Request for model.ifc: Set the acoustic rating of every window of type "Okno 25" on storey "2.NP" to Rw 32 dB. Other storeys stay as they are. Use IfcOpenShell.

First a look at what the model holds.

```python
import ifcopenshell
import ifcopenshell.util.element

model = ifcopenshell.open("model.ifc")
print(model.schema)
storey = next(s for s in model.by_type("IfcBuildingStorey") if s.Name == "2.NP")
windows = [e for e in ifcopenshell.util.element.get_decomposition(storey) if e.is_a("IfcWindow")]
seen = {}
for e in windows:
    element_type = ifcopenshell.util.element.get_type(e)
    key = (element_type.Name if element_type != e and element_type else None, ifcopenshell.util.element.get_pset(e, "Pset_WindowCommon", "AcousticRating"))
    seen[key] = seen.get(key, 0) + 1
for (name, value), count in sorted(seen.items(), key=str):
    print(count, "x", name, "|", value)
```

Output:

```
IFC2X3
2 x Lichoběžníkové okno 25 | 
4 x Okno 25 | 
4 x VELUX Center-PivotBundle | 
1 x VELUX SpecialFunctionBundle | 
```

```python
import ifcopenshell
import ifcopenshell.api.pset
import ifcopenshell.util.element

model = ifcopenshell.open("model.ifc")

storey = next(s for s in model.by_type("IfcBuildingStorey") if s.Name == "2.NP")
windows = [e for e in ifcopenshell.util.element.get_decomposition(storey) if e.is_a("IfcWindow")]

count = 0
for e in windows:
    element_type = ifcopenshell.util.element.get_type(e)
    if element_type in (None, e) or element_type.Name != "Okno 25":
        continue
    # add_pset returns the element's existing set when there is one.
    pset = ifcopenshell.api.pset.add_pset(model, product=e, name="Pset_WindowCommon")
    ifcopenshell.api.pset.edit_pset(model, pset=pset, properties={"AcousticRating": "Rw 32 dB"})
    count += 1

print(count, "windows updated")

model.write("model_rev.ifc")
```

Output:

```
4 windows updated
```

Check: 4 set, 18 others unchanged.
